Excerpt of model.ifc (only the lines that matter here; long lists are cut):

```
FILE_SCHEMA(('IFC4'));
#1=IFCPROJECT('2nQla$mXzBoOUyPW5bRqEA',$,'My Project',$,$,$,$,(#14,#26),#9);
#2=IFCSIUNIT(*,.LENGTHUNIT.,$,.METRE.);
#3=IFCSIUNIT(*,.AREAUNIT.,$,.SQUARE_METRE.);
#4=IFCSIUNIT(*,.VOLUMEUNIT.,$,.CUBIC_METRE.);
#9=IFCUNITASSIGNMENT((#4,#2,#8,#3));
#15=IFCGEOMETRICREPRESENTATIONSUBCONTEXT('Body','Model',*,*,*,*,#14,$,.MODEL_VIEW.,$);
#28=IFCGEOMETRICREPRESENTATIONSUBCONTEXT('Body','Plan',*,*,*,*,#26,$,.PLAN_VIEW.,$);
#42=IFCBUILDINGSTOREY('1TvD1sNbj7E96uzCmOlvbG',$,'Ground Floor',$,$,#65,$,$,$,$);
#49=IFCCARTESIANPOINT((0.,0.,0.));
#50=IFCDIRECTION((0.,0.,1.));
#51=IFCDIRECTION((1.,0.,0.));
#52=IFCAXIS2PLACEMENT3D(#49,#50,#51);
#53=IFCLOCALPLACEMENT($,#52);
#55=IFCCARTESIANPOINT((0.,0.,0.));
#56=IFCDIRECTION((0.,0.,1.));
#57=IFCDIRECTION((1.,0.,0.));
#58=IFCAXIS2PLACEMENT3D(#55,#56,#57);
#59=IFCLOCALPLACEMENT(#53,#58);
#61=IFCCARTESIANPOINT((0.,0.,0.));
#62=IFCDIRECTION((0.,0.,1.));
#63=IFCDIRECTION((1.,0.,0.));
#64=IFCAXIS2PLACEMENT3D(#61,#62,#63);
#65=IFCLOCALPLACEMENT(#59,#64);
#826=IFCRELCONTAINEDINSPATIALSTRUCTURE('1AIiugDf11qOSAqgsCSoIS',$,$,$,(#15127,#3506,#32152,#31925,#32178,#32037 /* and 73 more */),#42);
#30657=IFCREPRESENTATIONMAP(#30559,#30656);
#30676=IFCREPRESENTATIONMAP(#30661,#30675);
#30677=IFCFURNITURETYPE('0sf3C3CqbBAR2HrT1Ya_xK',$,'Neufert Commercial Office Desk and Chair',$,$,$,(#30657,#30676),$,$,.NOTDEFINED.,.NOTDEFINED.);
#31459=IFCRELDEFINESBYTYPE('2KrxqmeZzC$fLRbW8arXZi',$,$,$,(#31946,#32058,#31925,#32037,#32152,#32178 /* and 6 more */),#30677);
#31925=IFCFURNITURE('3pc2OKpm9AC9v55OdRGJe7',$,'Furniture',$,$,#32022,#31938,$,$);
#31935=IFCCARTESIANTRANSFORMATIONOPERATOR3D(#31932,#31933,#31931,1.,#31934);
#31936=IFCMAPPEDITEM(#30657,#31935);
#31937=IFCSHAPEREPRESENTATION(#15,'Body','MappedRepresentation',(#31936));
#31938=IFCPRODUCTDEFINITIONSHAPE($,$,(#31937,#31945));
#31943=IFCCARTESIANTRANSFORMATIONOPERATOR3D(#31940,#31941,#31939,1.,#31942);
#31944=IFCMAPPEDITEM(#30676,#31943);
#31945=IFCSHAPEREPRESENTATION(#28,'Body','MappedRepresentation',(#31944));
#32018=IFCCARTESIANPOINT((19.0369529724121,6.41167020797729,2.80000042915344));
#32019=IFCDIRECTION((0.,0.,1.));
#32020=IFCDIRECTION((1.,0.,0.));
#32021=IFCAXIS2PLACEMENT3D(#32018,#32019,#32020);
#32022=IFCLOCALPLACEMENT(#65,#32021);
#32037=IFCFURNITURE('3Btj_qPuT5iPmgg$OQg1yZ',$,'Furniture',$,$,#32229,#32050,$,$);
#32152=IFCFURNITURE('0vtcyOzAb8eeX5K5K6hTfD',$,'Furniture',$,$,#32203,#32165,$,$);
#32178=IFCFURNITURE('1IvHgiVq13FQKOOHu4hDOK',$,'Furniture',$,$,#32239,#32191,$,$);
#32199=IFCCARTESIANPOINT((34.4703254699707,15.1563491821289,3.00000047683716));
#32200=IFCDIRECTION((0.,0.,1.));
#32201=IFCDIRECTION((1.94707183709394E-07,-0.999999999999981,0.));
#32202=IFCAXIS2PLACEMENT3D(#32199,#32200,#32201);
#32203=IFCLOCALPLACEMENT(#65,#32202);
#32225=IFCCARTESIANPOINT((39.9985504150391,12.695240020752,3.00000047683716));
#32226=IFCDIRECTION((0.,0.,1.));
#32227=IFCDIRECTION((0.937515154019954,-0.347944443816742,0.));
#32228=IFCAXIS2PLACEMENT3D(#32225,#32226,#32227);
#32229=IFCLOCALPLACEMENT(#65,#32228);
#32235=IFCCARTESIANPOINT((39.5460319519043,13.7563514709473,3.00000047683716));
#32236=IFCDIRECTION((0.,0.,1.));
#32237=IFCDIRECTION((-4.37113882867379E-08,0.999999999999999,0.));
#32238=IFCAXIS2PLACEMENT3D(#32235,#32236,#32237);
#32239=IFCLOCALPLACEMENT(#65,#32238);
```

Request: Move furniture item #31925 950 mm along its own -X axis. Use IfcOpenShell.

```python
import ifcopenshell
import ifcopenshell.api.geometry
import ifcopenshell.util.placement
import ifcopenshell.util.unit

model = ifcopenshell.open("model.ifc")
unit_scale = ifcopenshell.util.unit.calculate_unit_scale(model)

item = model.by_guid("3pc2OKpm9AC9v55OdRGJe7")
matrix = ifcopenshell.util.placement.get_local_placement(item.ObjectPlacement)
matrix[:3, 3] -= matrix[:3, 0] * 0.95 / unit_scale
ifcopenshell.api.geometry.edit_object_placement(model, product=item, matrix=matrix, is_si=False)

print(ifcopenshell.util.placement.get_local_placement(item.ObjectPlacement).round(3) + 0.0)

model.write("model-out.ifc")
```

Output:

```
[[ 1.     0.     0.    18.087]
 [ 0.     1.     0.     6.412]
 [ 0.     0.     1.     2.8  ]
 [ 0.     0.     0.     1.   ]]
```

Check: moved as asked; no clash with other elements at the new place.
